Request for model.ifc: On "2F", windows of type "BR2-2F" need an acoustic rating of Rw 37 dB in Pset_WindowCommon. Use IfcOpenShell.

First a look at what the model holds.

```python
import ifcopenshell
import ifcopenshell.util.element

model = ifcopenshell.open("model.ifc")
print(model.schema)
storey = next(s for s in model.by_type("IfcBuildingStorey") if s.Name == "2F")
windows = [e for e in ifcopenshell.util.element.get_decomposition(storey) if e.is_a("IfcWindow")]
seen = {}
for e in windows:
    element_type = ifcopenshell.util.element.get_type(e)
    key = (element_type.Name if element_type != e and element_type else None, ifcopenshell.util.element.get_pset(e, "Pset_WindowCommon", "AcousticRating"))
    seen[key] = seen.get(key, 0) + 1
for (name, value), count in sorted(seen.items(), key=str):
    print(count, "x", name, "|", value)
```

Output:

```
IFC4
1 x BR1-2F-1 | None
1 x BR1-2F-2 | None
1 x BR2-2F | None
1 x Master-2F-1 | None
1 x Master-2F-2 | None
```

```python
import ifcopenshell
import ifcopenshell.api.pset
import ifcopenshell.util.element

model = ifcopenshell.open("model.ifc")

storey = next(s for s in model.by_type("IfcBuildingStorey") if s.Name == "2F")
windows = [e for e in ifcopenshell.util.element.get_decomposition(storey) if e.is_a("IfcWindow")]

count = 0
for e in windows:
    element_type = ifcopenshell.util.element.get_type(e)
    if element_type in (None, e) or element_type.Name != "BR2-2F":
        continue
    # add_pset returns the element's existing set when there is one.
    pset = ifcopenshell.api.pset.add_pset(model, product=e, name="Pset_WindowCommon")
    ifcopenshell.api.pset.edit_pset(model, pset=pset, properties={"AcousticRating": "Rw 37 dB"})
    count += 1

print(count, "windows updated")

model.write("model_v2.ifc")
```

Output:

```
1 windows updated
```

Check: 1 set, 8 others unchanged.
